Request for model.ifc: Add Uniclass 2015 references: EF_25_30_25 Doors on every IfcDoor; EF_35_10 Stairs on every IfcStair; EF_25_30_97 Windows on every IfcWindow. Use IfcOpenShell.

First a look at what the model holds.

```python
import ifcopenshell

model = ifcopenshell.open("model.ifc")
print(model.schema)
print("classifications:", [c.Name for c in model.by_type("IfcClassification")])
for ifc_class in ("IfcDoor", "IfcRoof", "IfcStair", "IfcWall", "IfcWindow"):
    print(ifc_class, len(model.by_type(ifc_class)))
```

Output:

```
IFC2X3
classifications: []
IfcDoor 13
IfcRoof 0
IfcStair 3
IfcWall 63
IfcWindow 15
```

```python
import ifcopenshell
import ifcopenshell.api.classification

model = ifcopenshell.open("model.ifc")

# IFC2X3 requires Source and Edition and has no link from the project to the system.
system = model.create_entity("IfcClassification", Source="NBS", Edition="2015", Name="Uniclass 2015")

codes = {
    "IfcDoor": ("EF_25_30_25", "Doors"),
    "IfcStair": ("EF_35_10", "Stairs"),
    "IfcWindow": ("EF_25_30_97", "Windows"),
}
for ifc_class, (code, name) in codes.items():
    products = model.by_type(ifc_class)
    ifcopenshell.api.classification.add_reference(
        model, products=products, classification=system, identification=code, name=name
    )
    print(code, len(products))

model.write("model_updated.ifc")
```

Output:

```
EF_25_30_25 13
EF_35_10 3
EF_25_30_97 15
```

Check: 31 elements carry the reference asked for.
